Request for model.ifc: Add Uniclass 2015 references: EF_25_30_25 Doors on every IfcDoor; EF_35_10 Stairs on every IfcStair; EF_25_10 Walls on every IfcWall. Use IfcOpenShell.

First a look at what the model holds.

```python
import ifcopenshell

model = ifcopenshell.open("model.ifc")
print(model.schema)
print("classifications:", [c.Name for c in model.by_type("IfcClassification")])
for ifc_class in ("IfcDoor", "IfcRoof", "IfcStair", "IfcWall", "IfcWindow"):
    print(ifc_class, len(model.by_type(ifc_class)))
```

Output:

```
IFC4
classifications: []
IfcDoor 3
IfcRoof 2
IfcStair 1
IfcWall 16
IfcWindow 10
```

```python
import ifcopenshell
import ifcopenshell.api.classification

model = ifcopenshell.open("model.ifc")

system = ifcopenshell.api.classification.add_classification(model, classification="Uniclass 2015")

codes = {
    "IfcDoor": ("EF_25_30_25", "Doors"),
    "IfcStair": ("EF_35_10", "Stairs"),
    "IfcWall": ("EF_25_10", "Walls"),
}
for ifc_class, (code, name) in codes.items():
    products = model.by_type(ifc_class)
    ifcopenshell.api.classification.add_reference(
        model, products=products, classification=system, identification=code, name=name
    )
    print(code, len(products))

model.write("model_updated.ifc")
```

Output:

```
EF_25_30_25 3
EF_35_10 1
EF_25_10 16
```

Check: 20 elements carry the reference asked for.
